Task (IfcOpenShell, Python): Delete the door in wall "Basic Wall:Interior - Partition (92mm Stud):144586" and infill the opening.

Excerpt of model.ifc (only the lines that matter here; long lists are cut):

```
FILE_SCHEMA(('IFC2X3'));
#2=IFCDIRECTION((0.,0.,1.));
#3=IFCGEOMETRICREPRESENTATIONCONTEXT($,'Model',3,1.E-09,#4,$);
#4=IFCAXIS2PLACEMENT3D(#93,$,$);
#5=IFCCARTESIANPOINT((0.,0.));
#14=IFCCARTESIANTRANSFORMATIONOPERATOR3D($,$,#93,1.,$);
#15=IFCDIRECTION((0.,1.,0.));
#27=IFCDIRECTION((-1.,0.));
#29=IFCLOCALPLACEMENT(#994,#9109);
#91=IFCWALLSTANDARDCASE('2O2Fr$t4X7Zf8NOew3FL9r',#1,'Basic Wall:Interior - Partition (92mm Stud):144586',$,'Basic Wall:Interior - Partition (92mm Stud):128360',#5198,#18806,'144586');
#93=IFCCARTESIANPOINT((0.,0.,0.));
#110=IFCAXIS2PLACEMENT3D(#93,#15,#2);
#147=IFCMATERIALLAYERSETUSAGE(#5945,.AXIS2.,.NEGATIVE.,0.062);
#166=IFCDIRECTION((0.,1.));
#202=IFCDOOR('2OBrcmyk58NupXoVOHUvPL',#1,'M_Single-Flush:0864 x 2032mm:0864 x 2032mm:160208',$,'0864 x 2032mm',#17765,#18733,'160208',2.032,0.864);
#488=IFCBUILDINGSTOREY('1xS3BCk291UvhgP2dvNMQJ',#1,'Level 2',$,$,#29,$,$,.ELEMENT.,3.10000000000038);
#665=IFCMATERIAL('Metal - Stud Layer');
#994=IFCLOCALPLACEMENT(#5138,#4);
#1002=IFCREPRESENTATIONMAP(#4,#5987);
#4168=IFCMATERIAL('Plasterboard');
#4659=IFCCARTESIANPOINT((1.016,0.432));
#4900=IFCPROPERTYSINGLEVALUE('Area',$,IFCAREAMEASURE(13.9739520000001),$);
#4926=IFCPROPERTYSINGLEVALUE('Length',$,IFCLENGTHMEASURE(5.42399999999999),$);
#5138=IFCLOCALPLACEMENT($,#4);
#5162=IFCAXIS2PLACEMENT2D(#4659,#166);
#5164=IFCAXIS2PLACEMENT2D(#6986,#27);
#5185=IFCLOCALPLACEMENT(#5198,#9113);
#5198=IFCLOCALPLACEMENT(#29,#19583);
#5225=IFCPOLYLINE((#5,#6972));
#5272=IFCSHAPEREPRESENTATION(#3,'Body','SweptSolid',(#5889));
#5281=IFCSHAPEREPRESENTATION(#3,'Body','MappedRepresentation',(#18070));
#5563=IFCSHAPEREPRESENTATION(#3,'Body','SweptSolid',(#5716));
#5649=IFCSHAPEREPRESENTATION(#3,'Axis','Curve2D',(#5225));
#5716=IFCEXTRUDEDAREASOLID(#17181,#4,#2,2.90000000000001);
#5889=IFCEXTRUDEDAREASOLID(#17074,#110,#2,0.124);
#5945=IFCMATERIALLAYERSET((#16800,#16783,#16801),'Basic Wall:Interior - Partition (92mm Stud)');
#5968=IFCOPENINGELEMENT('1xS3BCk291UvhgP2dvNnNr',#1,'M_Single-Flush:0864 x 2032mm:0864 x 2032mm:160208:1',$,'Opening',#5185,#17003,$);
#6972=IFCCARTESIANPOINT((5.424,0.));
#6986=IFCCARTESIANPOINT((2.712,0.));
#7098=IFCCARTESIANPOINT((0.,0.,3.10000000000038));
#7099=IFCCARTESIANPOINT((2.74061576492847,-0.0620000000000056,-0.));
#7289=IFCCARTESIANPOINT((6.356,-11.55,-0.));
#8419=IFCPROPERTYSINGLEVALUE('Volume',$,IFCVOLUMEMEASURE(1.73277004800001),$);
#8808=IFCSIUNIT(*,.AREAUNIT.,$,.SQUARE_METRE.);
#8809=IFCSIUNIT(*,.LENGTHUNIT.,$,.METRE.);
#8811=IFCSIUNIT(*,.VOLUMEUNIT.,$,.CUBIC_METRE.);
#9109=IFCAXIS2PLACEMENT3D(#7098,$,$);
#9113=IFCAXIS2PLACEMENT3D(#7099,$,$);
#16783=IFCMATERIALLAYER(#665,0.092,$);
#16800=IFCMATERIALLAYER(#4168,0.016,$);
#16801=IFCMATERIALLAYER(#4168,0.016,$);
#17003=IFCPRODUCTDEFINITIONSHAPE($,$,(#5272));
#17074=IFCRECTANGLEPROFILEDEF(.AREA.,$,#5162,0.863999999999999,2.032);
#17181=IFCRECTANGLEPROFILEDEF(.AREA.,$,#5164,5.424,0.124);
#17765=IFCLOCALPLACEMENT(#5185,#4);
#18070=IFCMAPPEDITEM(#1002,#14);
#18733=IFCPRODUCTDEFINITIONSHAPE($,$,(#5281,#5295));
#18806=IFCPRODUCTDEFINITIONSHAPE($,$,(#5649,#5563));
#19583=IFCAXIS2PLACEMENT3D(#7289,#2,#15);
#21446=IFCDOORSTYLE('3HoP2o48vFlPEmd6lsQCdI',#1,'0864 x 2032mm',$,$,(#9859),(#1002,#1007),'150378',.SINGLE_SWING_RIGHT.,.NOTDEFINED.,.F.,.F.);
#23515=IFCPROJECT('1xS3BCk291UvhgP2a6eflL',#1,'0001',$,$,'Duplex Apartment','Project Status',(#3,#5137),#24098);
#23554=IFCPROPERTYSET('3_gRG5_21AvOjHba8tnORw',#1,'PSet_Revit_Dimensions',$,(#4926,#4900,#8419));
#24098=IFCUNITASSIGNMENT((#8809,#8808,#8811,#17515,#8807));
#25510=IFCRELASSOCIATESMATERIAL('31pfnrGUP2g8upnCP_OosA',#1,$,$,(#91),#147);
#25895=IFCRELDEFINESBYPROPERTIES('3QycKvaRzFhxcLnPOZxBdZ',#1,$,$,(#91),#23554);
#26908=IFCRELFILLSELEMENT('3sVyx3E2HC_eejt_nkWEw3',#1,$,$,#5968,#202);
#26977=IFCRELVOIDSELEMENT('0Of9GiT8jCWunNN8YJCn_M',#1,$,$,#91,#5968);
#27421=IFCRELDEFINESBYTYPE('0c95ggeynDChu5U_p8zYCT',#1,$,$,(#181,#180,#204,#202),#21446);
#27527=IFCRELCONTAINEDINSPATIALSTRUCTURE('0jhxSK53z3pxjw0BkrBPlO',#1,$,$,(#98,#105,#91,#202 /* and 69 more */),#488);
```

```python
import ifcopenshell
import ifcopenshell.api.feature
import ifcopenshell.api.pset
import ifcopenshell.api.root
import ifcopenshell.geom
import ifcopenshell.util.element
import ifcopenshell.util.shape
import ifcopenshell.util.unit

model = ifcopenshell.open("model.ifc")
area_scale = ifcopenshell.util.unit.calculate_unit_scale(model, "AREAUNIT")
volume_scale = ifcopenshell.util.unit.calculate_unit_scale(model, "VOLUMEUNIT")
settings = ifcopenshell.geom.settings()


def volume(element):
    """Net volume in cubic metres, openings subtracted."""
    shape = ifcopenshell.geom.create_shape(settings, element)
    return ifcopenshell.util.shape.get_volume(shape.geometry)


door = model.by_guid("2OBrcmyk58NupXoVOHUvPL")
opening = door.FillsVoids[0].RelatingOpeningElement
wall = opening.VoidsElements[0].RelatingBuildingElement
before = volume(wall)

ifcopenshell.api.root.remove_product(model, product=door)
ifcopenshell.api.feature.remove_feature(model, feature=opening)

after = volume(wall)
thickness = 0.124  # wall thickness in metres

# Update the wall's stored quantities.
pset = model.by_id(ifcopenshell.util.element.get_pset(wall, "PSet_Revit_Dimensions", should_inherit=False)["id"])
ifcopenshell.api.pset.edit_pset(model, pset=pset, properties={
    "Area": model.create_entity("IfcAreaMeasure", after / thickness / area_scale),
    "Volume": model.create_entity("IfcVolumeMeasure", after / volume_scale),
})

print(f"wall volume {before:.3f} -> {after:.3f} m3")

model.write("model-out.ifc")
```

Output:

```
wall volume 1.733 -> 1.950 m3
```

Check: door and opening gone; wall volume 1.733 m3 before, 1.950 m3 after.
